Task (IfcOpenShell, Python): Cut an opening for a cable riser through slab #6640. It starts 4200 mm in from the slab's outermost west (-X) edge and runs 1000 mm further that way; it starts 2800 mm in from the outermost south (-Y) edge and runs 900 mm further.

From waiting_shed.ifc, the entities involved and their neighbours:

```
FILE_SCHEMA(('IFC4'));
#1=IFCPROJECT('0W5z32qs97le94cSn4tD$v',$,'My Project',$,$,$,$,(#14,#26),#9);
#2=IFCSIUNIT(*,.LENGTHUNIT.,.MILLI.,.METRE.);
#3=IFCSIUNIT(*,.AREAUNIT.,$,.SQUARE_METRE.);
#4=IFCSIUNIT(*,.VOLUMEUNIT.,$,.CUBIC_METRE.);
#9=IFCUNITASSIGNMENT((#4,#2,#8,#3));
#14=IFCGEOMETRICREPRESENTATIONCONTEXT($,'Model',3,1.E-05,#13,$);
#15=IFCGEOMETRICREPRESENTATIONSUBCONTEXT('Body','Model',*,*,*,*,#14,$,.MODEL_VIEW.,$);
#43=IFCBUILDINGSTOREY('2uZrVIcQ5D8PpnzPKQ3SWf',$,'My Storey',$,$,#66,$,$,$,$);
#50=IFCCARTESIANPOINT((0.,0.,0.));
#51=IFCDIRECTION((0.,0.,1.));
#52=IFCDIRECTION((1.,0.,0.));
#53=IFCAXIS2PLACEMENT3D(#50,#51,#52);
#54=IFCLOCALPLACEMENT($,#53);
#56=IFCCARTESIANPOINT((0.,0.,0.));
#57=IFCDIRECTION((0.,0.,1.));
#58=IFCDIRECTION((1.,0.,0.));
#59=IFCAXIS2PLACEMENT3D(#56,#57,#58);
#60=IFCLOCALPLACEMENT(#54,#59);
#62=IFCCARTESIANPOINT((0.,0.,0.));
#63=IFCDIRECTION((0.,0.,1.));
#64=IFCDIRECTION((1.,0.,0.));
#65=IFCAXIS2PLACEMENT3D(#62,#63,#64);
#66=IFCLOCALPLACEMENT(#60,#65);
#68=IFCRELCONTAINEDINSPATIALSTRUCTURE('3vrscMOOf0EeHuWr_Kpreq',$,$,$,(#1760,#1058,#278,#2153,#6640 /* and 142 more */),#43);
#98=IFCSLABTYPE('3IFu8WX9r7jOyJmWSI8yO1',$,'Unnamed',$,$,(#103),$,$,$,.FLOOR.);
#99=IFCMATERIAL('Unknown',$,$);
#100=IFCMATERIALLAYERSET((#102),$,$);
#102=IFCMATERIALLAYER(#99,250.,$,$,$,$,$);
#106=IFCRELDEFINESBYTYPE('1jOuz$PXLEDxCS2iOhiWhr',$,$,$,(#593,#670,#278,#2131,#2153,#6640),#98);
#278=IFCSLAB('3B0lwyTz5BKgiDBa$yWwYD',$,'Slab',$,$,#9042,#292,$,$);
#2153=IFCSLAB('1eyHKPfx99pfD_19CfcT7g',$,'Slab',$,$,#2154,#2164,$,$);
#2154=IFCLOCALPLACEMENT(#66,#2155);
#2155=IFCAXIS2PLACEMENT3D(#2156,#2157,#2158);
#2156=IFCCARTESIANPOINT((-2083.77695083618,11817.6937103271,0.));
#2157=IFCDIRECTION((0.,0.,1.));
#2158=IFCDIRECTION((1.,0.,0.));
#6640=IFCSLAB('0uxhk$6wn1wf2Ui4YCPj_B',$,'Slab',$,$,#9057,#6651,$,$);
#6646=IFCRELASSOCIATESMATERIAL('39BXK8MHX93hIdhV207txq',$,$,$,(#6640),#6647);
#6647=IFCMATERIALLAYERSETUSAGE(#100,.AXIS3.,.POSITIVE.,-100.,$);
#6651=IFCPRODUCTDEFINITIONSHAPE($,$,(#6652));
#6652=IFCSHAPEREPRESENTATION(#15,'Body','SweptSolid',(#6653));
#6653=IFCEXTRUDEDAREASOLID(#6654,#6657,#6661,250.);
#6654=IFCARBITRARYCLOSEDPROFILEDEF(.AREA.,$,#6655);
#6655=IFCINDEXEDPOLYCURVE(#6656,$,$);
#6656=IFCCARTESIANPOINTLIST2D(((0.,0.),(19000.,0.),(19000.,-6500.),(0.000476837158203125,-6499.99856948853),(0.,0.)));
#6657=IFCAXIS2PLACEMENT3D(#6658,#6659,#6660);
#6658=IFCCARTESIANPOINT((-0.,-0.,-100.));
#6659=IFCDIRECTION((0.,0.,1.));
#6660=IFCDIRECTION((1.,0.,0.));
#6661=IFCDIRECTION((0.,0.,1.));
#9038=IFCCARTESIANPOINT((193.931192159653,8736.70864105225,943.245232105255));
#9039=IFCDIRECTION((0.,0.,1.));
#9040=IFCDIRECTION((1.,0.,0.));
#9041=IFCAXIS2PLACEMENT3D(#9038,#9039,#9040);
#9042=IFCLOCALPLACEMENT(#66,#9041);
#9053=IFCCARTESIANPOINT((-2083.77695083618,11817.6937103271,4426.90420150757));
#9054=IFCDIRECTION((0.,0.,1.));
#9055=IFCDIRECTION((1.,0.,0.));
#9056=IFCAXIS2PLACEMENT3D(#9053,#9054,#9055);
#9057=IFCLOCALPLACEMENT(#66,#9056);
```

```python
import numpy as np
import ifcopenshell
import ifcopenshell.api.feature
import ifcopenshell.api.geometry
import ifcopenshell.api.root
import ifcopenshell.geom
import ifcopenshell.util.placement
import ifcopenshell.util.representation
import ifcopenshell.util.shape
import ifcopenshell.util.unit

model = ifcopenshell.open("waiting_shed.ifc")
unit_scale = ifcopenshell.util.unit.calculate_unit_scale(model)
settings = ifcopenshell.geom.settings()


def volume(element):
    """Net volume in cubic metres, openings subtracted."""
    shape = ifcopenshell.geom.create_shape(settings, element)
    return ifcopenshell.util.shape.get_volume(shape.geometry)


slab = model.by_id(6640)
before = volume(slab)

# Extent in the slab's own axes, in metres. The edges named are its -X and -Y sides.
slab_shape = ifcopenshell.geom.create_shape(settings, slab)
vertices = ifcopenshell.util.shape.get_vertices(slab_shape.geometry)
x_min, y_min, bottom = vertices.min(axis=0)
top = vertices[:, 2].max()

opening = ifcopenshell.api.root.create_entity(model, ifc_class="IfcOpeningElement", name="Cable riser opening", predefined_type="OPENING")
context = ifcopenshell.util.representation.get_context(model, "Model", "Body", "MODEL_VIEW")
width, depth = 1, 0.9
outline = [(0.0, 0.0), (width, 0.0), (width, depth), (0.0, depth), (0.0, 0.0)]
# Overshoot both faces by 50 mm so the cut is clean.
shape = ifcopenshell.api.geometry.add_slab_representation(
    model, context=context, depth=top - bottom + 0.1, polyline=outline
)
ifcopenshell.api.geometry.assign_representation(model, product=opening, representation=shape)

matrix = ifcopenshell.util.placement.get_local_placement(slab.ObjectPlacement)
matrix[:, 3] = matrix @ np.append(np.array([x_min + 4.2, y_min + 2.8, bottom - 0.05]) / unit_scale, 1.0)
ifcopenshell.api.geometry.edit_object_placement(model, product=opening, matrix=matrix, is_si=False)
ifcopenshell.api.feature.add_feature(model, feature=opening, element=slab)

after = volume(slab)

print(f"slab volume {before:.3f} -> {after:.3f} m3")

model.write("waiting_shed_v2.ifc")
```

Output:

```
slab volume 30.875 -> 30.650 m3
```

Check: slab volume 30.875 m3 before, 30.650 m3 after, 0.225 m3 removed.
